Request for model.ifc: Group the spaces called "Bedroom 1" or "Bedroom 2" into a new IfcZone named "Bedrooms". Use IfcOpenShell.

First a look at what the model holds.

```python
import ifcopenshell

model = ifcopenshell.open("model.ifc")
print(model.schema)
seen = {}
for space in model.by_type("IfcSpace"):
    seen[space.LongName] = seen.get(space.LongName, 0) + 1
for name, count in sorted(seen.items(), key=str):
    print(count, "x", name)
print("zones:", [z.Name for z in model.by_type("IfcZone")][:20])
```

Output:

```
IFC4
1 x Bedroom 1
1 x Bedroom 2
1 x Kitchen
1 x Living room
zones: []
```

```python
import ifcopenshell
import ifcopenshell.api.group
import ifcopenshell.api.root

model = ifcopenshell.open("model.ifc")

names = {"Bedroom 1", "Bedroom 2"}
spaces = [s for s in model.by_type("IfcSpace") if s.LongName in names]

zone = ifcopenshell.api.root.create_entity(model, ifc_class="IfcZone", name="Bedrooms")
ifcopenshell.api.group.assign_group(model, products=spaces, group=zone)
print(len(spaces), "spaces in", zone.Name)

model.write("model_edited.ifc")
```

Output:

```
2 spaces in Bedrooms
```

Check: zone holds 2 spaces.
